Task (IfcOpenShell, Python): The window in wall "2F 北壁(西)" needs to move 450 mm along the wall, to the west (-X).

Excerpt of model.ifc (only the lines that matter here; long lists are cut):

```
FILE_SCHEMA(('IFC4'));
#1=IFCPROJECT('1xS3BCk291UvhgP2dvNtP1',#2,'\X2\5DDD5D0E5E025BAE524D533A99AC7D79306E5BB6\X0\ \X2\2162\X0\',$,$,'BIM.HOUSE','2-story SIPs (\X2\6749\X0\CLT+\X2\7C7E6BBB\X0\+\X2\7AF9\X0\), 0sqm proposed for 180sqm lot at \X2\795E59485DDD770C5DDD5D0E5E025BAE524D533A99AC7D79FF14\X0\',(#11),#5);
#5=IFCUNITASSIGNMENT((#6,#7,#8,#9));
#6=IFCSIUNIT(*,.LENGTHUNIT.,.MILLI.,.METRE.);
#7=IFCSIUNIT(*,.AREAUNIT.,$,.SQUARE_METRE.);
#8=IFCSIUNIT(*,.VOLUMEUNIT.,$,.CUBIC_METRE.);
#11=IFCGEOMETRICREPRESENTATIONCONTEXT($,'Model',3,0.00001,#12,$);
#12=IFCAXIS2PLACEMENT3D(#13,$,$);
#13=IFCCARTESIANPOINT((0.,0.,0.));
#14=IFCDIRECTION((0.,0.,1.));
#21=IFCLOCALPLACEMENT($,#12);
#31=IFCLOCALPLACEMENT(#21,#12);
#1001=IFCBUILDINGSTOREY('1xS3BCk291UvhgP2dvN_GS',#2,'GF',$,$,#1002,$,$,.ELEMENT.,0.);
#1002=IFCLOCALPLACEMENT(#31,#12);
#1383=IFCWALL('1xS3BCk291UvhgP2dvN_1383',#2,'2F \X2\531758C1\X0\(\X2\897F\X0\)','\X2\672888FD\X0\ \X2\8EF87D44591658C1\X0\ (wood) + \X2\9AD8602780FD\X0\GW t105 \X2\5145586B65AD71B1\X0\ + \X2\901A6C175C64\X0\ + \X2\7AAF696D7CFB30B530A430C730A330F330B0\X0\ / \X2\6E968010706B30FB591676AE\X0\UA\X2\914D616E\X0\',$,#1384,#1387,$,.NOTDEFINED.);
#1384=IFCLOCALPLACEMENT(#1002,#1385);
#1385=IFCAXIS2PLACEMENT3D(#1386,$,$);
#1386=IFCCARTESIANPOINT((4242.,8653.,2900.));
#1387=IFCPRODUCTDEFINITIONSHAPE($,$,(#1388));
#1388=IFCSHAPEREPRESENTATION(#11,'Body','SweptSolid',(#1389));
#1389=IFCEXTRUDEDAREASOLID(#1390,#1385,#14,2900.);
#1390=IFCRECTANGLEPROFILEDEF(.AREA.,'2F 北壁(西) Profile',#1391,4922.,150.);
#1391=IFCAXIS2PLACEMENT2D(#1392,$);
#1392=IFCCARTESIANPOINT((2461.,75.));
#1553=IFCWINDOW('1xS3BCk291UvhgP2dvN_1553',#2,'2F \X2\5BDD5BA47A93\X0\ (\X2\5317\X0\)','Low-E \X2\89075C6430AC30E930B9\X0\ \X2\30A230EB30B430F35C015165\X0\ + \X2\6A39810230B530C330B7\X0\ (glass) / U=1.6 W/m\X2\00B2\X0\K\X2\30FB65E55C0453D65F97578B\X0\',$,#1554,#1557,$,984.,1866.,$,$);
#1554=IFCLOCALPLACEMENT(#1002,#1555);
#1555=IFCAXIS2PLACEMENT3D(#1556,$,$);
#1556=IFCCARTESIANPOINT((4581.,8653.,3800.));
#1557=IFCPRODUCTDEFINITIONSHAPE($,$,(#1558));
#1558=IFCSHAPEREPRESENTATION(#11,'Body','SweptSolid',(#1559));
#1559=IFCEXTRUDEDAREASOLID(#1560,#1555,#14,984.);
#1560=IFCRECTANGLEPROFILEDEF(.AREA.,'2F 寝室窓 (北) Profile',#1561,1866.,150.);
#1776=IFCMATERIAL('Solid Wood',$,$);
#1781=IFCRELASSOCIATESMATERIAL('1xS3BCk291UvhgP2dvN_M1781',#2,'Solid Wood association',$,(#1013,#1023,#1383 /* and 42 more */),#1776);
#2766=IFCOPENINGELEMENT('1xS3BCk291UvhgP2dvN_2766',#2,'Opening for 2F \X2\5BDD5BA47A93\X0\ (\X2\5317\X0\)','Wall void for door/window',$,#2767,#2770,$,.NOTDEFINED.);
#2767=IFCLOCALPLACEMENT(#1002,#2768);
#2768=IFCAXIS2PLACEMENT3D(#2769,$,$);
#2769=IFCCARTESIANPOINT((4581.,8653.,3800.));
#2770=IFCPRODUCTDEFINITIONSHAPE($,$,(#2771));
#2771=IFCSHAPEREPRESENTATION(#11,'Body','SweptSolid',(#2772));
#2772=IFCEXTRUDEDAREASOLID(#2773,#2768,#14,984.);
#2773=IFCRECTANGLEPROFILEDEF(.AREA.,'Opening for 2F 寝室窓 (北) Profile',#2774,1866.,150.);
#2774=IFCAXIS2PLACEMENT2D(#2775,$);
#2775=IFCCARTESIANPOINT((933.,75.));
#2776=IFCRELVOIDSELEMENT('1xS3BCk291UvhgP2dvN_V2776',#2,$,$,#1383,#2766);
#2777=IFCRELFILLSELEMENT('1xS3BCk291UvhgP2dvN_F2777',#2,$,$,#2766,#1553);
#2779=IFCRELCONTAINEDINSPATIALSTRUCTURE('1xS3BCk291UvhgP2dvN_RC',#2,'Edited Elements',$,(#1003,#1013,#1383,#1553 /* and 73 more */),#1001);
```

```python
import ifcopenshell
import ifcopenshell.api.geometry
import ifcopenshell.util.placement
import ifcopenshell.util.unit

model = ifcopenshell.open("model.ifc")
unit_scale = ifcopenshell.util.unit.calculate_unit_scale(model)

window = model.by_guid("1xS3BCk291UvhgP2dvN_1553")
opening = window.FillsVoids[0].RelatingOpeningElement
wall = opening.VoidsElements[0].RelatingBuildingElement

wall_matrix = ifcopenshell.util.placement.get_local_placement(wall.ObjectPlacement)
shift = wall_matrix[:3, 0] * -0.45 / unit_scale
before = ifcopenshell.util.placement.get_local_placement(window.ObjectPlacement)[:3, 3].copy()

# The window is not placed relative to its opening, so move both.
for product in (opening, window):
    matrix = ifcopenshell.util.placement.get_local_placement(product.ObjectPlacement)
    matrix[:3, 3] += shift
    ifcopenshell.api.geometry.edit_object_placement(model, product=product, matrix=matrix, is_si=False)

after = ifcopenshell.util.placement.get_local_placement(window.ObjectPlacement)[:3, 3]
print("window moved by", (after - before).round(3) + 0.0)

model.write("model_updated.ifc")
```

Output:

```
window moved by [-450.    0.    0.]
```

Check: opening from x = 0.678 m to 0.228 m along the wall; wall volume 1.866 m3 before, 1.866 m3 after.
